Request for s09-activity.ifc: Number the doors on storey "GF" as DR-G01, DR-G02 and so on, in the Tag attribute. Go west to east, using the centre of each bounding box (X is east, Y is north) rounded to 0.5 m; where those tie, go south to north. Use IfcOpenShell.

First a look at what the model holds.

```python
import ifcopenshell
import ifcopenshell.util.element
import ifcopenshell.util.placement

model = ifcopenshell.open("s09-activity.ifc")
print(model.schema)
storey = next(s for s in model.by_type("IfcBuildingStorey") if s.Name == "GF")
doors = [e for e in ifcopenshell.util.element.get_decomposition(storey) if e.is_a("IfcDoor")]
for e in sorted(doors, key=lambda e: e.id()):
    origin = ifcopenshell.util.placement.get_local_placement(e.ObjectPlacement)[:3, 3]
    print(e.id(), e.Tag, e.Name, origin.round(2) + 0.0, sep=" | ")
```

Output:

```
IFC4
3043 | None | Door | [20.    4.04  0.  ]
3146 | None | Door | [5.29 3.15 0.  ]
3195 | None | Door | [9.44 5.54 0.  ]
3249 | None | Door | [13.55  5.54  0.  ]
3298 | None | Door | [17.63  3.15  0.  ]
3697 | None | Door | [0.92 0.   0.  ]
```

```python
import ifcopenshell
import ifcopenshell.geom
import ifcopenshell.util.element
import ifcopenshell.util.shape

model = ifcopenshell.open("s09-activity.ifc")
settings = ifcopenshell.geom.settings()
settings.set("use-world-coords", True)


def centre(element):
    shape = ifcopenshell.geom.create_shape(settings, element)
    return ifcopenshell.util.shape.get_bbox_centroid(shape.geometry)


storey = next(s for s in model.by_type("IfcBuildingStorey") if s.Name == "GF")
doors = [e for e in ifcopenshell.util.element.get_decomposition(storey) if e.is_a("IfcDoor")]

# Insertion points can sit at a corner or the storey origin, so sort by the geometry (in metres).
centres = {e: centre(e) for e in doors}
doors.sort(key=lambda e: (round(centres[e][0] / 0.5), centres[e][1]))

for i, e in enumerate(doors, start=1):
    number = f"DR-G{i:02d}"
    e.Tag = number
    print(e.id(), number)

model.write("s09-activity_v2.ifc")
```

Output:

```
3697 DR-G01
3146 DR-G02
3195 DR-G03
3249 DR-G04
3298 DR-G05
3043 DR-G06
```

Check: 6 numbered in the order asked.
